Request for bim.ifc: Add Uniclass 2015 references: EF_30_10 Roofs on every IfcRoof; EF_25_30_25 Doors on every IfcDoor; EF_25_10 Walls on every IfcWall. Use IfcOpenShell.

First a look at what the model holds.

```python
import ifcopenshell

model = ifcopenshell.open("bim.ifc")
print(model.schema)
print("classifications:", [c.Name for c in model.by_type("IfcClassification")])
for ifc_class in ("IfcDoor", "IfcRoof", "IfcStair", "IfcWall", "IfcWindow"):
    print(ifc_class, len(model.by_type(ifc_class)))
```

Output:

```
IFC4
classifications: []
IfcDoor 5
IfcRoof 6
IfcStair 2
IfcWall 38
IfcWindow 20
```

```python
import ifcopenshell
import ifcopenshell.api.classification

model = ifcopenshell.open("bim.ifc")

system = ifcopenshell.api.classification.add_classification(model, classification="Uniclass 2015")

codes = {
    "IfcRoof": ("EF_30_10", "Roofs"),
    "IfcDoor": ("EF_25_30_25", "Doors"),
    "IfcWall": ("EF_25_10", "Walls"),
}
for ifc_class, (code, name) in codes.items():
    products = model.by_type(ifc_class)
    ifcopenshell.api.classification.add_reference(
        model, products=products, classification=system, identification=code, name=name
    )
    print(code, len(products))

model.write("bim_rev.ifc")
```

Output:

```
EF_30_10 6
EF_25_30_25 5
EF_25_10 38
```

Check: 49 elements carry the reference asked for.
